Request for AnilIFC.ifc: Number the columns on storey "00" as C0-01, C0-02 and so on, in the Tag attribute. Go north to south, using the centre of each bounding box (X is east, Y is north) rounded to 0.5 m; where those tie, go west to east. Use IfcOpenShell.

First a look at what the model holds.

```python
import ifcopenshell
import ifcopenshell.util.element
import ifcopenshell.util.placement

model = ifcopenshell.open("AnilIFC.ifc")
print(model.schema)
storey = next(s for s in model.by_type("IfcBuildingStorey") if s.Name == "00")
columns = [e for e in ifcopenshell.util.element.get_decomposition(storey) if e.is_a("IfcColumn")]
for e in sorted(columns, key=lambda e: e.id()):
    origin = ifcopenshell.util.placement.get_local_placement(e.ObjectPlacement)[:3, 3]
    print(e.id(), e.Tag, e.Name, origin.round(2) + 0.0, sep=" | ")
```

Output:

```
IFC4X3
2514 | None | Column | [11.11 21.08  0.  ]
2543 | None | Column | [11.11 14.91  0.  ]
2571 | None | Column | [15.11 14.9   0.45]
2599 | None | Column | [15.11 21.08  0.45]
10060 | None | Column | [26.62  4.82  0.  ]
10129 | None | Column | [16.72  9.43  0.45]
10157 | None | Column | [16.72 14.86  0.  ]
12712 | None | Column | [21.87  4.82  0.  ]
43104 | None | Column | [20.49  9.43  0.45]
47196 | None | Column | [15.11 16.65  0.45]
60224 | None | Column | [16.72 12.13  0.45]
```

```python
import ifcopenshell
import ifcopenshell.geom
import ifcopenshell.util.element
import ifcopenshell.util.shape

model = ifcopenshell.open("AnilIFC.ifc")
settings = ifcopenshell.geom.settings()
settings.set("use-world-coords", True)


def centre(element):
    shape = ifcopenshell.geom.create_shape(settings, element)
    return ifcopenshell.util.shape.get_bbox_centroid(shape.geometry)


storey = next(s for s in model.by_type("IfcBuildingStorey") if s.Name == "00")
columns = [e for e in ifcopenshell.util.element.get_decomposition(storey) if e.is_a("IfcColumn")]

# Insertion points can sit at a corner or the storey origin, so sort by the geometry (in metres).
centres = {e: centre(e) for e in columns}
columns.sort(key=lambda e: (-round(centres[e][1] / 0.5), centres[e][0]))

for i, e in enumerate(columns, start=1):
    number = f"C0-{i:02d}"
    e.Tag = number
    print(e.id(), number)

model.write("AnilIFC_rev.ifc")
```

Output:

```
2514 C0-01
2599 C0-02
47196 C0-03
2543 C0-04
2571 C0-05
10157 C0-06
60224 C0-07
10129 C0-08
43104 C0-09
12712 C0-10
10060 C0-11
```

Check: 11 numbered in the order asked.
